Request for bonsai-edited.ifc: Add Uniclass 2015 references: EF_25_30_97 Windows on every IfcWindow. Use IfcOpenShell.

First a look at what the model holds.

```python
import ifcopenshell

model = ifcopenshell.open("bonsai-edited.ifc")
print(model.schema)
print("classifications:", [c.Name for c in model.by_type("IfcClassification")])
for ifc_class in ("IfcDoor", "IfcRoof", "IfcStair", "IfcWall", "IfcWindow"):
    print(ifc_class, len(model.by_type(ifc_class)))
```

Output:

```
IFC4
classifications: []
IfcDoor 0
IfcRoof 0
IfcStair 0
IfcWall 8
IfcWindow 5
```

```python
import ifcopenshell
import ifcopenshell.api.classification

model = ifcopenshell.open("bonsai-edited.ifc")

system = ifcopenshell.api.classification.add_classification(model, classification="Uniclass 2015")

codes = {
    "IfcWindow": ("EF_25_30_97", "Windows"),
}
for ifc_class, (code, name) in codes.items():
    products = model.by_type(ifc_class)
    ifcopenshell.api.classification.add_reference(
        model, products=products, classification=system, identification=code, name=name
    )
    print(code, len(products))

model.write("bonsai-edited_updated.ifc")
```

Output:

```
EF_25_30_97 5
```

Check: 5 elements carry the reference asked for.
